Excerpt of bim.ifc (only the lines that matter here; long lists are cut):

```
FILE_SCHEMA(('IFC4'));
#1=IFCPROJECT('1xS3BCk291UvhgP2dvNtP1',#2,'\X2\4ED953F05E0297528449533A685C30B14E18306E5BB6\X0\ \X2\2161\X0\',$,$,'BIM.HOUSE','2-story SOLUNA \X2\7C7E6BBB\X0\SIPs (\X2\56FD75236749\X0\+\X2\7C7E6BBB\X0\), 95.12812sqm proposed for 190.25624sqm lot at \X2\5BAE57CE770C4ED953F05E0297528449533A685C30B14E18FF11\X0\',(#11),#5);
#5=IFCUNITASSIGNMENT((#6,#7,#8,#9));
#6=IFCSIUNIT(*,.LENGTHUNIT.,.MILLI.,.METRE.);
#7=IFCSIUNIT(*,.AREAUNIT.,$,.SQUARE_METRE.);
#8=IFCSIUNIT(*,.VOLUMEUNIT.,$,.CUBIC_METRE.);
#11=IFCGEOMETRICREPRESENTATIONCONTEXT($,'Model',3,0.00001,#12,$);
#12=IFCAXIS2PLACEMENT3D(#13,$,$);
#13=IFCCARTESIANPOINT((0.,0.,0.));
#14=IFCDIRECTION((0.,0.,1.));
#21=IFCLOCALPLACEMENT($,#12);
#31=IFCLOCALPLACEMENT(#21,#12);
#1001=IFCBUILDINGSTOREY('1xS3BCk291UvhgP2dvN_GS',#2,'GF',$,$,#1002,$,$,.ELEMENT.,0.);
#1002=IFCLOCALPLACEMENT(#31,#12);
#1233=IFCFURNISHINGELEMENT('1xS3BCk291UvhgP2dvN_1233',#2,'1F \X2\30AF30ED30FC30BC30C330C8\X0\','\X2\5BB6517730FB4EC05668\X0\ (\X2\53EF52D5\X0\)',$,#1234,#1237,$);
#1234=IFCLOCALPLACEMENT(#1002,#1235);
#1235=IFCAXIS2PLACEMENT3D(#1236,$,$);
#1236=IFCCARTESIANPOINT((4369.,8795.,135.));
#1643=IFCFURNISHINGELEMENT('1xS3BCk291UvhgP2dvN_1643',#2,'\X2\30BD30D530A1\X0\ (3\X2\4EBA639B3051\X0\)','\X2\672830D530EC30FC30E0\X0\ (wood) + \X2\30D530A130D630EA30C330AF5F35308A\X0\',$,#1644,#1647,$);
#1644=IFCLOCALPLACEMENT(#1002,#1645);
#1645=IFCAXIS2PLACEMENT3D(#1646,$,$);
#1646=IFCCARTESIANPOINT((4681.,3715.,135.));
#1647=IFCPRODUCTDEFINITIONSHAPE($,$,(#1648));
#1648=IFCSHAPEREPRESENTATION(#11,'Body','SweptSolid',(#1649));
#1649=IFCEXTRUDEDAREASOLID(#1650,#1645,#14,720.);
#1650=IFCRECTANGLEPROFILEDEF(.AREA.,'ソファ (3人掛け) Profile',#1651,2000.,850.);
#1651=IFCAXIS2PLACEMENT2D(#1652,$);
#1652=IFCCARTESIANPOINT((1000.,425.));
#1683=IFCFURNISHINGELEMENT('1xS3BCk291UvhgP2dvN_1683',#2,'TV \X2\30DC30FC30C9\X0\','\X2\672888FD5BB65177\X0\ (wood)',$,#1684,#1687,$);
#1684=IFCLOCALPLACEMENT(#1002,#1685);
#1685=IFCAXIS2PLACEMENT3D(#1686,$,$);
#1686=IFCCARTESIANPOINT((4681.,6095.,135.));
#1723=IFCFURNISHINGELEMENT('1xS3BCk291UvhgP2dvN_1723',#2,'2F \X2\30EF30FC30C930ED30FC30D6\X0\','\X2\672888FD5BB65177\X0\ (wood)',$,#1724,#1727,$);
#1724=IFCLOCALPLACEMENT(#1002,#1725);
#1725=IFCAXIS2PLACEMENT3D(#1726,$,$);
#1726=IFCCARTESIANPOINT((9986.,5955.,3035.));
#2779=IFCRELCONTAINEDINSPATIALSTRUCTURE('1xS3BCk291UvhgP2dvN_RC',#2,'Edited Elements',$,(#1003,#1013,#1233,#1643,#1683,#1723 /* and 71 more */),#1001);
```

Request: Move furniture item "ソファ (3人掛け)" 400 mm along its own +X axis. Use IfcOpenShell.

```python
import ifcopenshell
import ifcopenshell.api.geometry
import ifcopenshell.util.placement

model = ifcopenshell.open("bim.ifc")

item = model.by_id(1643)
matrix = ifcopenshell.util.placement.get_local_placement(item.ObjectPlacement)
matrix[:3, 3] += matrix[:3, 0] * 400.0
ifcopenshell.api.geometry.edit_object_placement(model, product=item, matrix=matrix, is_si=False)

print(ifcopenshell.util.placement.get_local_placement(item.ObjectPlacement).round(3) + 0.0)

model.write("bim_updated.ifc")
```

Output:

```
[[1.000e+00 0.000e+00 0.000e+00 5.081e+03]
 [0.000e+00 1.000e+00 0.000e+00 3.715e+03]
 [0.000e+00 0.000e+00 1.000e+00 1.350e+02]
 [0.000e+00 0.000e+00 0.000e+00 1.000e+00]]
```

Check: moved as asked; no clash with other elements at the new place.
